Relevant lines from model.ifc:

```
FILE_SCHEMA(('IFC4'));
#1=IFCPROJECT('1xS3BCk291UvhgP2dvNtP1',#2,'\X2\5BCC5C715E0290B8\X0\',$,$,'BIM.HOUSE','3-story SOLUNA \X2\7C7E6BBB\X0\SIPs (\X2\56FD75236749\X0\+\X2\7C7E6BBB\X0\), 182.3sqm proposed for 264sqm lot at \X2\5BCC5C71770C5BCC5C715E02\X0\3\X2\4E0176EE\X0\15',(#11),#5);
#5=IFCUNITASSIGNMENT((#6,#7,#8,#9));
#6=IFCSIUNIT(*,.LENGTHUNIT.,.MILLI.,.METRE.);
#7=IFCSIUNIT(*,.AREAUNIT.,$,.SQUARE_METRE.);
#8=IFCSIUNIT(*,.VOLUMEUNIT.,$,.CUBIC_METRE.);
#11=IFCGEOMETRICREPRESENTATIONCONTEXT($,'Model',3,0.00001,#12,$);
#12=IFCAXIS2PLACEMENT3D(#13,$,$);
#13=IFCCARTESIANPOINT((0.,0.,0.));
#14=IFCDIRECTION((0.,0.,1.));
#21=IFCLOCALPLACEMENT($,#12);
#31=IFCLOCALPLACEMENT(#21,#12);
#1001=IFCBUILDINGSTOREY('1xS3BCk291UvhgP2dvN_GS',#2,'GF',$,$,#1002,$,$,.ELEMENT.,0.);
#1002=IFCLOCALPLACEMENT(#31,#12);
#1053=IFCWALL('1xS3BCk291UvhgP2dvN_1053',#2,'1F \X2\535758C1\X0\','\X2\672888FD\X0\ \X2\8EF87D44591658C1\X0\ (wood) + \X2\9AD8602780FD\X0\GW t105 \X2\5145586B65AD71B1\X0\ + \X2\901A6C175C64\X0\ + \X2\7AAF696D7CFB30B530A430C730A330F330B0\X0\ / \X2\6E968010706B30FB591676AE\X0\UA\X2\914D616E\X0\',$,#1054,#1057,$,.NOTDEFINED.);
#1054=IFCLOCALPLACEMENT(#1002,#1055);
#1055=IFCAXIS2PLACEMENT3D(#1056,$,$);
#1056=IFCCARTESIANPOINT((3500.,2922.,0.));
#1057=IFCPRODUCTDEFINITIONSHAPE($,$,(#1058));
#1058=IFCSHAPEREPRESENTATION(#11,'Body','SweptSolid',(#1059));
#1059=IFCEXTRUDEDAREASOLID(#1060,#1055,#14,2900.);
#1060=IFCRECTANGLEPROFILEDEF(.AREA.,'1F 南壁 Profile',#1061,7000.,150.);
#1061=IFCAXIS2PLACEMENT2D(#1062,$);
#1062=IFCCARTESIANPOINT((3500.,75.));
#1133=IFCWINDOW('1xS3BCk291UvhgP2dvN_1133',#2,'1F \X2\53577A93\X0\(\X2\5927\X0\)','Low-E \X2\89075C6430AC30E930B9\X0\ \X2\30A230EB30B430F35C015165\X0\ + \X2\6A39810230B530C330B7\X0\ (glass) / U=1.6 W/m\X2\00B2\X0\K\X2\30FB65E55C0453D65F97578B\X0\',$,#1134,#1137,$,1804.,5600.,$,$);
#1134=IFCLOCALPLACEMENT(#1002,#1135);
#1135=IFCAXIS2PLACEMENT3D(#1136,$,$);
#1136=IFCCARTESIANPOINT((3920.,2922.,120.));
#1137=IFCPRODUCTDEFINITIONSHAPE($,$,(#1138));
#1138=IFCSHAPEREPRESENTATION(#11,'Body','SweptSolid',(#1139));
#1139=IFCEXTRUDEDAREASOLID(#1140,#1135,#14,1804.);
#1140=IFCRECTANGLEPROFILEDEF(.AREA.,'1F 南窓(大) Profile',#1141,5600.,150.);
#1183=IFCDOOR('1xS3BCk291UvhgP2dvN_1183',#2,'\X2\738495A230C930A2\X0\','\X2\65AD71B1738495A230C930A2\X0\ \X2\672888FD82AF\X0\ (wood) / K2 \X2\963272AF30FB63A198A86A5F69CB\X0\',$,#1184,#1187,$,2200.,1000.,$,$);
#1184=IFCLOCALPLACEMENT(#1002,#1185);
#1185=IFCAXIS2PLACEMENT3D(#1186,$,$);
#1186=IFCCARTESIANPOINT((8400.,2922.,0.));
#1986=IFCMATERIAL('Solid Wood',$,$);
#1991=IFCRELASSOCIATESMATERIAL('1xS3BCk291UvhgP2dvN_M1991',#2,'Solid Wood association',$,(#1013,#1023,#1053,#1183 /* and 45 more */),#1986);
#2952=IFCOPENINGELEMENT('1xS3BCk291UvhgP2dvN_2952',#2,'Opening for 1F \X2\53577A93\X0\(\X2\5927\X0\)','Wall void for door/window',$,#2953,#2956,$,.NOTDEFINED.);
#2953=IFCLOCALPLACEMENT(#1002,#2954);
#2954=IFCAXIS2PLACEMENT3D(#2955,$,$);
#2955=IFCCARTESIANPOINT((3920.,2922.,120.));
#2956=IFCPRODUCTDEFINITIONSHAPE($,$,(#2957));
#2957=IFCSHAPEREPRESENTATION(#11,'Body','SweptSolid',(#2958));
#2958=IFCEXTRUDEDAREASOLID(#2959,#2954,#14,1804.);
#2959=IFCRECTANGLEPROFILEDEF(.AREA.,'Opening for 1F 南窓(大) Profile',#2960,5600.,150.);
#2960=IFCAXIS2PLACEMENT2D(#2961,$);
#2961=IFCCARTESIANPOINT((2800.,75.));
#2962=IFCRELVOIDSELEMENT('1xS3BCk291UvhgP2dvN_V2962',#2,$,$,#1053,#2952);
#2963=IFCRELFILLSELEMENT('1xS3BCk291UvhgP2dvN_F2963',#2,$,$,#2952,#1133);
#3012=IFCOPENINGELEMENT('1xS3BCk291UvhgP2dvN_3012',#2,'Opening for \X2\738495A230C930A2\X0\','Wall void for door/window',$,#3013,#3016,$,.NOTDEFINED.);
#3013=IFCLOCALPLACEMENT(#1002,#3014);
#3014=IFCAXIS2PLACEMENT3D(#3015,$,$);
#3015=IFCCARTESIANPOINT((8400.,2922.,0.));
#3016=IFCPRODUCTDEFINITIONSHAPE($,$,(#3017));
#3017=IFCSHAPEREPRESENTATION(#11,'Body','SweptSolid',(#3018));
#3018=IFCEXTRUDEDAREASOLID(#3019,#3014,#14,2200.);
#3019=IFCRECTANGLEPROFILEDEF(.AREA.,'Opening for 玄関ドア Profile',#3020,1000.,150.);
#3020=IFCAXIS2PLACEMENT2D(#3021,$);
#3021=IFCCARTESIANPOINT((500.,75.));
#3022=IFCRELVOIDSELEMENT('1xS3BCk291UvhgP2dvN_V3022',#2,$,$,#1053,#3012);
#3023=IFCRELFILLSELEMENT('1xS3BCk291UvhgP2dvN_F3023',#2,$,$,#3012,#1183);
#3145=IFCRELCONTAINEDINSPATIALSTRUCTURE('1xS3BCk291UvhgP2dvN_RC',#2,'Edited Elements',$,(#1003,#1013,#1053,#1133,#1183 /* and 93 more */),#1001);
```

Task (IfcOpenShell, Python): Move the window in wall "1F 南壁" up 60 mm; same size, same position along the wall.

```python
import numpy as np
import ifcopenshell
import ifcopenshell.api.geometry
import ifcopenshell.util.placement
import ifcopenshell.util.unit

model = ifcopenshell.open("model.ifc")
unit_scale = ifcopenshell.util.unit.calculate_unit_scale(model)

window = model.by_guid("1xS3BCk291UvhgP2dvN_1133")
opening = window.FillsVoids[0].RelatingOpeningElement
dz = 0.06 / unit_scale

shift = np.array([0.0, 0.0, dz])
# The window is not placed relative to its opening, so move both.
for product in (opening, window):
    matrix = ifcopenshell.util.placement.get_local_placement(product.ObjectPlacement)
    matrix[:3, 3] += shift
    ifcopenshell.api.geometry.edit_object_placement(model, product=product, matrix=matrix, is_si=False)

print(f"moved by {dz * unit_scale:+.3f} m")

model.write("model-out.ifc")
```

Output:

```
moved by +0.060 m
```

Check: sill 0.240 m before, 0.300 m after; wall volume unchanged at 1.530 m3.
